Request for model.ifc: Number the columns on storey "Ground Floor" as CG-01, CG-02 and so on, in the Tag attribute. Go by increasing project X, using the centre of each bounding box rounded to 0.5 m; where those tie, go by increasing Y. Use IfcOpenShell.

First a look at what the model holds.

```python
import ifcopenshell
import ifcopenshell.util.element
import ifcopenshell.util.placement

model = ifcopenshell.open("model.ifc")
print(model.schema)
storey = next(s for s in model.by_type("IfcBuildingStorey") if s.Name == "Ground Floor")
columns = [e for e in ifcopenshell.util.element.get_decomposition(storey) if e.is_a("IfcColumn")]
for e in sorted(columns, key=lambda e: e.id()):
    origin = ifcopenshell.util.placement.get_local_placement(e.ObjectPlacement)[:3, 3]
    print(e.id(), e.Tag, e.Name, origin.round(2) + 0.0, sep=" | ")
```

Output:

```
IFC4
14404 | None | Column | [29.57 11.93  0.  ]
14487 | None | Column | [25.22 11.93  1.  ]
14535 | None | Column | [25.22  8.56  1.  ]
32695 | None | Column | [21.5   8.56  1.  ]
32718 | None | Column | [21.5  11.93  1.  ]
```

```python
import ifcopenshell
import ifcopenshell.geom
import ifcopenshell.util.element
import ifcopenshell.util.shape

model = ifcopenshell.open("model.ifc")
settings = ifcopenshell.geom.settings()
settings.set("use-world-coords", True)


def centre(element):
    shape = ifcopenshell.geom.create_shape(settings, element)
    return ifcopenshell.util.shape.get_bbox_centroid(shape.geometry)


storey = next(s for s in model.by_type("IfcBuildingStorey") if s.Name == "Ground Floor")
columns = [e for e in ifcopenshell.util.element.get_decomposition(storey) if e.is_a("IfcColumn")]

# Insertion points can sit at a corner or the storey origin, so sort by the geometry (in metres).
centres = {e: centre(e) for e in columns}
columns.sort(key=lambda e: (round(centres[e][0] / 0.5), centres[e][1]))

for i, e in enumerate(columns, start=1):
    number = f"CG-{i:02d}"
    e.Tag = number
    print(e.id(), number)

model.write("model_rev.ifc")
```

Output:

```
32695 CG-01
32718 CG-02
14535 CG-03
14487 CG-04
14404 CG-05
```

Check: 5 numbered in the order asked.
